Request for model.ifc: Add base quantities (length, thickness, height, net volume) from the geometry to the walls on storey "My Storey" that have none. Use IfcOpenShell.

First a look at what the model holds.

```python
import ifcopenshell
import ifcopenshell.util.element
import ifcopenshell.util.unit

model = ifcopenshell.open("model.ifc")
print(model.schema)
for unit_type in ("LENGTHUNIT", "AREAUNIT", "VOLUMEUNIT"):
    print(unit_type, ifcopenshell.util.unit.calculate_unit_scale(model, unit_type))
storey = next(s for s in model.by_type("IfcBuildingStorey") if s.Name == "My Storey")
walls = [e for e in ifcopenshell.util.element.get_decomposition(storey) if e.is_a("IfcWall")]
for e in sorted(walls, key=lambda e: e.id()):
    print(e.id(), e.is_a(), e.Name, list(ifcopenshell.util.element.get_psets(e, qtos_only=True)), sep=" | ")
```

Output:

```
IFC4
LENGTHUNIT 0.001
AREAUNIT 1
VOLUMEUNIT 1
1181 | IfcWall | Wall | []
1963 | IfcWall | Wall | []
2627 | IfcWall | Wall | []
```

```python
import ifcopenshell
import ifcopenshell.api.pset
import ifcopenshell.geom
import ifcopenshell.util.element
import ifcopenshell.util.shape
import ifcopenshell.util.unit

model = ifcopenshell.open("model.ifc")
unit_scale = ifcopenshell.util.unit.calculate_unit_scale(model)
volume_scale = ifcopenshell.util.unit.calculate_unit_scale(model, "VOLUMEUNIT")
settings = ifcopenshell.geom.settings()

storey = next(s for s in model.by_type("IfcBuildingStorey") if s.Name == "My Storey")
walls = [e for e in ifcopenshell.util.element.get_decomposition(storey) if e.is_a("IfcWall")]

for e in sorted(walls, key=lambda e: e.id()):
    if ifcopenshell.util.element.get_psets(e, qtos_only=True, should_inherit=False):
        continue
    # Geometry comes back in metres, in the element's own axes.
    shape = ifcopenshell.geom.create_shape(settings, e)
    values = {
        "Length": ifcopenshell.util.shape.get_x(shape.geometry) / unit_scale,
        "Width": ifcopenshell.util.shape.get_y(shape.geometry) / unit_scale,
        "Height": ifcopenshell.util.shape.get_z(shape.geometry) / unit_scale,
        "NetVolume": ifcopenshell.util.shape.get_volume(shape.geometry) / volume_scale,
    }
    qto = ifcopenshell.api.pset.add_qto(model, product=e, name="Qto_WallBaseQuantities")
    ifcopenshell.api.pset.edit_qto(model, qto=qto, properties=values)
    print(e.id(), {k: round(v, 3) for k, v in values.items()})

model.write("model_rev.ifc")
```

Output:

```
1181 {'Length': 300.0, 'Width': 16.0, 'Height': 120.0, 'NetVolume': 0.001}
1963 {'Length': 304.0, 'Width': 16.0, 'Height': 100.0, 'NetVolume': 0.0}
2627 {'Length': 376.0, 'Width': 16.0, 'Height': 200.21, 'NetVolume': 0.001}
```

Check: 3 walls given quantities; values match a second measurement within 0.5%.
